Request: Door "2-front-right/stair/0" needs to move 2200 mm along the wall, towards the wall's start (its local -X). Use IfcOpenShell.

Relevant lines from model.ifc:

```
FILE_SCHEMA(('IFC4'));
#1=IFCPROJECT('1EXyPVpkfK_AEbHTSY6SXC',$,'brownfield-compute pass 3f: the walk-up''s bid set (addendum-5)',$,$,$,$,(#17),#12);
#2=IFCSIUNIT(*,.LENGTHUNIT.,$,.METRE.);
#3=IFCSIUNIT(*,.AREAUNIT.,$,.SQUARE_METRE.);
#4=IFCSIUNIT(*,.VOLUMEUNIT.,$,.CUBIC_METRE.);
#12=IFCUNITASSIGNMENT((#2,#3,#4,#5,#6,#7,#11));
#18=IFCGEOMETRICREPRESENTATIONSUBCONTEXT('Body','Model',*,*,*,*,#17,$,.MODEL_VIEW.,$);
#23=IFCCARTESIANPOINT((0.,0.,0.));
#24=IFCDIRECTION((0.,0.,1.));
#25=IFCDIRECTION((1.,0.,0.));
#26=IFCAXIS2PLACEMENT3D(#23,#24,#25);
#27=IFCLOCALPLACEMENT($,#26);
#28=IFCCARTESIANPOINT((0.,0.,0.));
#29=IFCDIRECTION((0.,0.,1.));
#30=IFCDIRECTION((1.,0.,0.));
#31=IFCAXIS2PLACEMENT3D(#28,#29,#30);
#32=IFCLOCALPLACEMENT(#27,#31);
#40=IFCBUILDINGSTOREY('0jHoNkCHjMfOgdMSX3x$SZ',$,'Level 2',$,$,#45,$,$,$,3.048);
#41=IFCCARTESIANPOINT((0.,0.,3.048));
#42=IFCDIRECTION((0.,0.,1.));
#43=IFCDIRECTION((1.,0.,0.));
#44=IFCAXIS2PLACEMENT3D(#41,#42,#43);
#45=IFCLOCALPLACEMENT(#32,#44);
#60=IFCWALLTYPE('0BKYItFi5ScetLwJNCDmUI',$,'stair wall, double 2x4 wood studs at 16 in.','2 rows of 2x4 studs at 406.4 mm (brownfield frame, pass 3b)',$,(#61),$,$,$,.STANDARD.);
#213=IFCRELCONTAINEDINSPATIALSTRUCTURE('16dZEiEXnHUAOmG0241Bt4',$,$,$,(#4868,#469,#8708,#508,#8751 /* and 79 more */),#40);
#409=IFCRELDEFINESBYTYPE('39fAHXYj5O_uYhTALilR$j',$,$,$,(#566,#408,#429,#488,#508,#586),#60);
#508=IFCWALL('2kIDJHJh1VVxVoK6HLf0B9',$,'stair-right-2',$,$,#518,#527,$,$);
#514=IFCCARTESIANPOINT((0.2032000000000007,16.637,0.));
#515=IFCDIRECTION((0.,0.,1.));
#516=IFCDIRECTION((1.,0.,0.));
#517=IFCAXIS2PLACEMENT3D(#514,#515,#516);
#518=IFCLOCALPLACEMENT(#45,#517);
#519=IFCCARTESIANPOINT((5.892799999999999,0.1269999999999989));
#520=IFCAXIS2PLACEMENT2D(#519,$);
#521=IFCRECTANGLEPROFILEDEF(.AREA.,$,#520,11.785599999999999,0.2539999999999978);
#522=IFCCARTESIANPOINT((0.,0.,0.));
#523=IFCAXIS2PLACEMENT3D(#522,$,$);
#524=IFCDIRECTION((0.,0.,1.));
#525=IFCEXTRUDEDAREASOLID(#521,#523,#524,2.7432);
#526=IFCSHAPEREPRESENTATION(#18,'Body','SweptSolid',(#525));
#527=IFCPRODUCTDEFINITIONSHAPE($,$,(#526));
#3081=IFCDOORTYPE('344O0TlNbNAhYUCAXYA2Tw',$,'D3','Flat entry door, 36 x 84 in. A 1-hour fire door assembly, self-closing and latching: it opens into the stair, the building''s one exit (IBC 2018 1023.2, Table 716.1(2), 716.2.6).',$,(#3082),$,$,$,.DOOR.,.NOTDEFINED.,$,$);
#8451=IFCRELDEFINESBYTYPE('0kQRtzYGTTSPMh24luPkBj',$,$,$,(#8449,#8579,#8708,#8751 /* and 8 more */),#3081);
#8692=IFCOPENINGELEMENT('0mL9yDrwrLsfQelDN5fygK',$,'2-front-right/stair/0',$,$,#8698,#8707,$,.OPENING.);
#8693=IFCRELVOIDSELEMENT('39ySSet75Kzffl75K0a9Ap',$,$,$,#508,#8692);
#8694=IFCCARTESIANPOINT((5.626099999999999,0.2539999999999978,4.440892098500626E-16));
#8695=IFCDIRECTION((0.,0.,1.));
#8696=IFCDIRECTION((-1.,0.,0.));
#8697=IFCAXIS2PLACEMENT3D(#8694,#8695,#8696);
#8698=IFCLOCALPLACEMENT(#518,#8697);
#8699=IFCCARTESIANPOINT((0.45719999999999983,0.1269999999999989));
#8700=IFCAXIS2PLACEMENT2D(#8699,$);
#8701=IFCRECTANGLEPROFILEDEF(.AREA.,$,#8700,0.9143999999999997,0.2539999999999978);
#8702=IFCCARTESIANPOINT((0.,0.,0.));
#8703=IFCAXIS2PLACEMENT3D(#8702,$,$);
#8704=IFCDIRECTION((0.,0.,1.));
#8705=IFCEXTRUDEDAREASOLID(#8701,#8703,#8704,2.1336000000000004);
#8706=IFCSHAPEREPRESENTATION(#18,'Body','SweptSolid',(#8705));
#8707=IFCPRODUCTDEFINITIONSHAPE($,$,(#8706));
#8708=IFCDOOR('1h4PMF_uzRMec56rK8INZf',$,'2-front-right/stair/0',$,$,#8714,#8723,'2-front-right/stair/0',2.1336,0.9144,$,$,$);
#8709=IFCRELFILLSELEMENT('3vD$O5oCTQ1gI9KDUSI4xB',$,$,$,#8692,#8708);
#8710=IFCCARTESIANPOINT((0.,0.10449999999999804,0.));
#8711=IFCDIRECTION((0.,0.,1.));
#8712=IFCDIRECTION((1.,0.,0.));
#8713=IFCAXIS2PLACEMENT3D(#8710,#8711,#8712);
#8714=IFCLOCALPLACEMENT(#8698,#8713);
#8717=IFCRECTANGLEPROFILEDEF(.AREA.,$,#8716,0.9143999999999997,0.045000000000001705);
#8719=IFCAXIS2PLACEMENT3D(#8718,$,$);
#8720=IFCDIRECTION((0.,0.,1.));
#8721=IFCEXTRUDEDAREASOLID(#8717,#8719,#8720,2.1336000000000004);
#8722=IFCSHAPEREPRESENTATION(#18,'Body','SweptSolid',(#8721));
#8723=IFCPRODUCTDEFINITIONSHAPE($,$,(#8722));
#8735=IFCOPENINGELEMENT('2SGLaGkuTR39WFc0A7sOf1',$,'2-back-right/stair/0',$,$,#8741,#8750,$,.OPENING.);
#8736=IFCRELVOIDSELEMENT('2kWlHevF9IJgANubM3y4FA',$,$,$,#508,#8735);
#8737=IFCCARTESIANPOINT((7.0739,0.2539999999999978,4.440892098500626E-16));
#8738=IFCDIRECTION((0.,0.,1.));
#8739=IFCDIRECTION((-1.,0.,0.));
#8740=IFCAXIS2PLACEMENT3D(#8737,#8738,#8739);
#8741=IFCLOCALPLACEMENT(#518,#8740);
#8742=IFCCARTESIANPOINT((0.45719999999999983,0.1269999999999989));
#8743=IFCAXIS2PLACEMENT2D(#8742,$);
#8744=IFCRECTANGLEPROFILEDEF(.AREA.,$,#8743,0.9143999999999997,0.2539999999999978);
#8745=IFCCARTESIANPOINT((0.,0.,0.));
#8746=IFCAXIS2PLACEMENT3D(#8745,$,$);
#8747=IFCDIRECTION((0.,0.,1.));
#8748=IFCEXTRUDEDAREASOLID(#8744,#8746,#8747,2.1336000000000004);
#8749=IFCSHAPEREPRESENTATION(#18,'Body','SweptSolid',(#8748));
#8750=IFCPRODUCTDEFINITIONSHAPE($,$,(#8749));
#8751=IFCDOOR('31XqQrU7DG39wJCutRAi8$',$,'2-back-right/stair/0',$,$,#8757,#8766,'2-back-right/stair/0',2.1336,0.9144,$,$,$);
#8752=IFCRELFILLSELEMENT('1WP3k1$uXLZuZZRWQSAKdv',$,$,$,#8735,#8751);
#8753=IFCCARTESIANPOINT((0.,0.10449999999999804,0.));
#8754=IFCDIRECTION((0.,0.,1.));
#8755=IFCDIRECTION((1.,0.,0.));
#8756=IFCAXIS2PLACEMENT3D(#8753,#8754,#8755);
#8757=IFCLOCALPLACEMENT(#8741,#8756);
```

```python
import ifcopenshell
import ifcopenshell.api.geometry
import ifcopenshell.util.placement
import ifcopenshell.util.unit

model = ifcopenshell.open("model.ifc")
unit_scale = ifcopenshell.util.unit.calculate_unit_scale(model)

door = model.by_guid("1h4PMF_uzRMec56rK8INZf")
opening = door.FillsVoids[0].RelatingOpeningElement
wall = opening.VoidsElements[0].RelatingBuildingElement

wall_matrix = ifcopenshell.util.placement.get_local_placement(wall.ObjectPlacement)
shift = wall_matrix[:3, 0] * -2.2 / unit_scale
before = ifcopenshell.util.placement.get_local_placement(door.ObjectPlacement)[:3, 3].copy()

# The door is placed relative to its opening, so it follows when the opening moves.
matrix = ifcopenshell.util.placement.get_local_placement(opening.ObjectPlacement)
matrix[:3, 3] += shift
ifcopenshell.api.geometry.edit_object_placement(
    model, product=opening, matrix=matrix, is_si=False, should_transform_children=True
)

after = ifcopenshell.util.placement.get_local_placement(door.ObjectPlacement)[:3, 3]
print("door moved by", (after - before).round(3) + 0.0)

model.write("model_updated.ifc")
```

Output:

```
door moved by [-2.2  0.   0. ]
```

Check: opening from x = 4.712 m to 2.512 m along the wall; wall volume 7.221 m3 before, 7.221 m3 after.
